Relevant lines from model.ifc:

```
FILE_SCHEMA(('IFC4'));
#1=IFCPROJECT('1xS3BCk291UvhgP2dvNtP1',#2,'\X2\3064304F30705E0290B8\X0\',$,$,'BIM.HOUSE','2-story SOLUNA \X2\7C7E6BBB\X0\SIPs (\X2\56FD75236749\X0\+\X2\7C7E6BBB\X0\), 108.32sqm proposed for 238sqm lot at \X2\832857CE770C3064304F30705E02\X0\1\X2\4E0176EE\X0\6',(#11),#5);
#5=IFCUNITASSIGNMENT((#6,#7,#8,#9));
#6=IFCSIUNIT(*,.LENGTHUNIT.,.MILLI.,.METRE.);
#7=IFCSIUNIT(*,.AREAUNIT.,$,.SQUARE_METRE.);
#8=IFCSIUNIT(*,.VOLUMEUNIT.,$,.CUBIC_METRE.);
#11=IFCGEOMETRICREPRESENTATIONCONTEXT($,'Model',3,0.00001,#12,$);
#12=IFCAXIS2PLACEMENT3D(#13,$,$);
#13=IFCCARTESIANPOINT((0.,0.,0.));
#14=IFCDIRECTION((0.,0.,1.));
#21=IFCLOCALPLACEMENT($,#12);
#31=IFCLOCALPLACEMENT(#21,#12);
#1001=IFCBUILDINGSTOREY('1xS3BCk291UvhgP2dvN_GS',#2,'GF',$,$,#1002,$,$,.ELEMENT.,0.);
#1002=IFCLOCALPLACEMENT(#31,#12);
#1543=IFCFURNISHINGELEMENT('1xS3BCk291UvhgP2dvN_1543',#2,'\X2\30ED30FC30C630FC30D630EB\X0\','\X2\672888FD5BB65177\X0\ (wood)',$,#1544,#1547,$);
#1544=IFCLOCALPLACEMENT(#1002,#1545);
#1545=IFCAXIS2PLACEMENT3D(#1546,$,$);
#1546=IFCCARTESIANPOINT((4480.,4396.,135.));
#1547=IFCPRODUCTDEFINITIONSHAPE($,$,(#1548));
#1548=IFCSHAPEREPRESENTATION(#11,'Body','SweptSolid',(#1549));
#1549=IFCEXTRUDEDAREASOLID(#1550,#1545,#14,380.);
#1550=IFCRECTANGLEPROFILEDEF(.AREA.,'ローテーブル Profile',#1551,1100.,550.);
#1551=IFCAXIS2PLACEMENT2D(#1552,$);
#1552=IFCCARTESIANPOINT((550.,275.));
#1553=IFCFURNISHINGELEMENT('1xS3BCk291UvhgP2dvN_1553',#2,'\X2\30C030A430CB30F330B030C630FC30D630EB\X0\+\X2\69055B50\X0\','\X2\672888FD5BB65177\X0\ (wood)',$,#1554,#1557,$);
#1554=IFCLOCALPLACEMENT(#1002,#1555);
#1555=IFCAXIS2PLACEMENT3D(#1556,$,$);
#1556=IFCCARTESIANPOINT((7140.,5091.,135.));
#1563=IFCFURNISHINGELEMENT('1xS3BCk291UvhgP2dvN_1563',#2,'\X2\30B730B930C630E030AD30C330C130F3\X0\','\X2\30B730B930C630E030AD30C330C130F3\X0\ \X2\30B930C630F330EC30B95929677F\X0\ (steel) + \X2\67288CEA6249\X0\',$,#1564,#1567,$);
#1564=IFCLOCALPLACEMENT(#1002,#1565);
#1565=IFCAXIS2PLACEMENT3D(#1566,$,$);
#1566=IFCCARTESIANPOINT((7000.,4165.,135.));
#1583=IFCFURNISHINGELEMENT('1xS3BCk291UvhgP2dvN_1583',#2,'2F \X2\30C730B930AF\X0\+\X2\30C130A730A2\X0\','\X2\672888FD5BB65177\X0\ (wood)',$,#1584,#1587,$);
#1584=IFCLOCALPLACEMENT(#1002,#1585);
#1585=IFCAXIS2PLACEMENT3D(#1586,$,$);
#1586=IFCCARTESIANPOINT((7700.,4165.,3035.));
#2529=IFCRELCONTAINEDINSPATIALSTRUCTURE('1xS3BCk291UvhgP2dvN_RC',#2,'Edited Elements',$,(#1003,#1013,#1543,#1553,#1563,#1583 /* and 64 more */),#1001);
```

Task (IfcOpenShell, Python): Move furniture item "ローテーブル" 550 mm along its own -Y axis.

```python
import ifcopenshell
import ifcopenshell.api.geometry
import ifcopenshell.util.placement

model = ifcopenshell.open("model.ifc")

item = model.by_id(1543)
matrix = ifcopenshell.util.placement.get_local_placement(item.ObjectPlacement)
matrix[:3, 3] -= matrix[:3, 1] * 550.0
ifcopenshell.api.geometry.edit_object_placement(model, product=item, matrix=matrix, is_si=False)

print(ifcopenshell.util.placement.get_local_placement(item.ObjectPlacement).round(3) + 0.0)

model.write("model-out.ifc")
```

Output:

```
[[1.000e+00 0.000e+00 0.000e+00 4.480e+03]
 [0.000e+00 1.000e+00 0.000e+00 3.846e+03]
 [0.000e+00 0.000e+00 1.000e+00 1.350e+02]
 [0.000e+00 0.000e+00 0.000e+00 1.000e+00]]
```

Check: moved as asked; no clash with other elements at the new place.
